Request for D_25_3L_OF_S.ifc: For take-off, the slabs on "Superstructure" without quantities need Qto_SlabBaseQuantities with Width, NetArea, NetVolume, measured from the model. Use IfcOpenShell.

First a look at what the model holds.

```python
import ifcopenshell
import ifcopenshell.util.element
import ifcopenshell.util.unit

model = ifcopenshell.open("D_25_3L_OF_S.ifc")
print(model.schema)
for unit_type in ("LENGTHUNIT", "AREAUNIT", "VOLUMEUNIT"):
    print(unit_type, ifcopenshell.util.unit.calculate_unit_scale(model, unit_type))
storey = next(s for s in model.by_type("IfcBuildingStorey") if s.Name == "Superstructure")
slabs = [e for e in ifcopenshell.util.element.get_decomposition(storey) if e.is_a("IfcSlab")]
for e in sorted(slabs, key=lambda e: e.id()):
    print(e.id(), e.is_a(), e.Name, list(ifcopenshell.util.element.get_psets(e, qtos_only=True)), sep=" | ")
```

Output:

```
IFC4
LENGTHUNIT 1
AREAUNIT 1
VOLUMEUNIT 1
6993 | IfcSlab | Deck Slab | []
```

```python
import ifcopenshell
import ifcopenshell.api.pset
import ifcopenshell.geom
import ifcopenshell.util.element
import ifcopenshell.util.shape
import ifcopenshell.util.unit

model = ifcopenshell.open("D_25_3L_OF_S.ifc")
unit_scale = ifcopenshell.util.unit.calculate_unit_scale(model)
area_scale = ifcopenshell.util.unit.calculate_unit_scale(model, "AREAUNIT")
volume_scale = ifcopenshell.util.unit.calculate_unit_scale(model, "VOLUMEUNIT")
settings = ifcopenshell.geom.settings()

storey = next(s for s in model.by_type("IfcBuildingStorey") if s.Name == "Superstructure")
slabs = [e for e in ifcopenshell.util.element.get_decomposition(storey) if e.is_a("IfcSlab")]

for e in sorted(slabs, key=lambda e: e.id()):
    if ifcopenshell.util.element.get_psets(e, qtos_only=True, should_inherit=False):
        continue
    # Geometry comes back in metres, in the element's own axes.
    shape = ifcopenshell.geom.create_shape(settings, e)
    values = {
        "Width": ifcopenshell.util.shape.get_z(shape.geometry) / unit_scale,
        "NetArea": ifcopenshell.util.shape.get_footprint_area(shape.geometry) / area_scale,
        "NetVolume": ifcopenshell.util.shape.get_volume(shape.geometry) / volume_scale,
    }
    qto = ifcopenshell.api.pset.add_qto(model, product=e, name="Qto_SlabBaseQuantities")
    ifcopenshell.api.pset.edit_qto(model, qto=qto, properties=values)
    print(e.id(), {k: round(v, 3) for k, v in values.items()})

model.write("D_25_3L_OF_S-out.ifc")
```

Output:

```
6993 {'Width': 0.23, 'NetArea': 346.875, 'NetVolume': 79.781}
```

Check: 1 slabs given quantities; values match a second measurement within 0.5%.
